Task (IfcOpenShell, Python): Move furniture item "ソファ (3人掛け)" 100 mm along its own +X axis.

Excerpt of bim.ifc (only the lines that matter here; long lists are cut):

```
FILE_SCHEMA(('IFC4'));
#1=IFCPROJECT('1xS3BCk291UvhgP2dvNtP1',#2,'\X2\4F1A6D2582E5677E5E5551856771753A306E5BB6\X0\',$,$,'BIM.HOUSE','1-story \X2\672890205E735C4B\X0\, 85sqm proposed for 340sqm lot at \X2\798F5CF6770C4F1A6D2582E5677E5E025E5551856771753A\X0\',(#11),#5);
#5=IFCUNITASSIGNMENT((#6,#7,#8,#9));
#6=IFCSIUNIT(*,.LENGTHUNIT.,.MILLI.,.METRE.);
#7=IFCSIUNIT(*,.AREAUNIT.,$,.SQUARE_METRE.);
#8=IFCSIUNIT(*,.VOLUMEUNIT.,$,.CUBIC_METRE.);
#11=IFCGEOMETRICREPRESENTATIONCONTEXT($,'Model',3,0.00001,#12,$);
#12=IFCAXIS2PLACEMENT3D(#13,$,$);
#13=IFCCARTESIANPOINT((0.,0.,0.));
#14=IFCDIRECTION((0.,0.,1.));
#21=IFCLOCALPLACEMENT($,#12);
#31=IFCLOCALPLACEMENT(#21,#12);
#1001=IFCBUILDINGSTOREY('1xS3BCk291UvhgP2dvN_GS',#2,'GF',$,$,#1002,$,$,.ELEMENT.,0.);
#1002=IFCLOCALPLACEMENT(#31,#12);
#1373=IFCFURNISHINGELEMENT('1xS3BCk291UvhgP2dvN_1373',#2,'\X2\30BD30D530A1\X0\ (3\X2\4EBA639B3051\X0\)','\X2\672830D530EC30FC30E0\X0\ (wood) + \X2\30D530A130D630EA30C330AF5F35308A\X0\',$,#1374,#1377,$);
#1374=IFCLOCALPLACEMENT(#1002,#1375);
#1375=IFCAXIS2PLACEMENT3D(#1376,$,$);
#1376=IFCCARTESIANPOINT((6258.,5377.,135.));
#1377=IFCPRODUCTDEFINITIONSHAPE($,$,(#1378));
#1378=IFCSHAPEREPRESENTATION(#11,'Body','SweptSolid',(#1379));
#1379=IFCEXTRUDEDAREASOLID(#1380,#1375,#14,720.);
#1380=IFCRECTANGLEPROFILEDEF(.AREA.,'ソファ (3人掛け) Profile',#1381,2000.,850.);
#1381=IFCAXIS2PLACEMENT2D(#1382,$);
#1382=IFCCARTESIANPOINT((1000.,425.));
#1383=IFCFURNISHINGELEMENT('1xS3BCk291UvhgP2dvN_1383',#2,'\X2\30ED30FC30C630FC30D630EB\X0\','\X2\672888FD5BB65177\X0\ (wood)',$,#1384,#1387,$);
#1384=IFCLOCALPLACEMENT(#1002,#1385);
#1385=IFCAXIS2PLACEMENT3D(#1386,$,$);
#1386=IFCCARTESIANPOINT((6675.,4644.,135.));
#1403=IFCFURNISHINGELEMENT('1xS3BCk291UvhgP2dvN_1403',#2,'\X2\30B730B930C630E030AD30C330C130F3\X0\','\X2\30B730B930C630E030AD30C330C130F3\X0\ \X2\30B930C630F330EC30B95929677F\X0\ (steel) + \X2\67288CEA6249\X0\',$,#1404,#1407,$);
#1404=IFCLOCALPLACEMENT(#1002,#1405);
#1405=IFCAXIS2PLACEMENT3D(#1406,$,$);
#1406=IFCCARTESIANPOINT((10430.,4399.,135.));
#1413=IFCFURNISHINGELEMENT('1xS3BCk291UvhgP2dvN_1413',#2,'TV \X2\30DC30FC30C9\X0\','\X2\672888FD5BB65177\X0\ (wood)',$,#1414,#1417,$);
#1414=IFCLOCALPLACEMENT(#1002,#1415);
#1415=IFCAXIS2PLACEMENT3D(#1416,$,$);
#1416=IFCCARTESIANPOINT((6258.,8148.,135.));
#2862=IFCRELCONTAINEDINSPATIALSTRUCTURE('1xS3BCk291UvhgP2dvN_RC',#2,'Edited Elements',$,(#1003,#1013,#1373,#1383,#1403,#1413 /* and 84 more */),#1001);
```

```python
import ifcopenshell
import ifcopenshell.api.geometry
import ifcopenshell.util.placement

model = ifcopenshell.open("bim.ifc")

item = model.by_guid("1xS3BCk291UvhgP2dvN_1373")
matrix = ifcopenshell.util.placement.get_local_placement(item.ObjectPlacement)
matrix[:3, 3] += matrix[:3, 0] * 100.0
ifcopenshell.api.geometry.edit_object_placement(model, product=item, matrix=matrix, is_si=False)

print(ifcopenshell.util.placement.get_local_placement(item.ObjectPlacement).round(3) + 0.0)

model.write("bim_v2.ifc")
```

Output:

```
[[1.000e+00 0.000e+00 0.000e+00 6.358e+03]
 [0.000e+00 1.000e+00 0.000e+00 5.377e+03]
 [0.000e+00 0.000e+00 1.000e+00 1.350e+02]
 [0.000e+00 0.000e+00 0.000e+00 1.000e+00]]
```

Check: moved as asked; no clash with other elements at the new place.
